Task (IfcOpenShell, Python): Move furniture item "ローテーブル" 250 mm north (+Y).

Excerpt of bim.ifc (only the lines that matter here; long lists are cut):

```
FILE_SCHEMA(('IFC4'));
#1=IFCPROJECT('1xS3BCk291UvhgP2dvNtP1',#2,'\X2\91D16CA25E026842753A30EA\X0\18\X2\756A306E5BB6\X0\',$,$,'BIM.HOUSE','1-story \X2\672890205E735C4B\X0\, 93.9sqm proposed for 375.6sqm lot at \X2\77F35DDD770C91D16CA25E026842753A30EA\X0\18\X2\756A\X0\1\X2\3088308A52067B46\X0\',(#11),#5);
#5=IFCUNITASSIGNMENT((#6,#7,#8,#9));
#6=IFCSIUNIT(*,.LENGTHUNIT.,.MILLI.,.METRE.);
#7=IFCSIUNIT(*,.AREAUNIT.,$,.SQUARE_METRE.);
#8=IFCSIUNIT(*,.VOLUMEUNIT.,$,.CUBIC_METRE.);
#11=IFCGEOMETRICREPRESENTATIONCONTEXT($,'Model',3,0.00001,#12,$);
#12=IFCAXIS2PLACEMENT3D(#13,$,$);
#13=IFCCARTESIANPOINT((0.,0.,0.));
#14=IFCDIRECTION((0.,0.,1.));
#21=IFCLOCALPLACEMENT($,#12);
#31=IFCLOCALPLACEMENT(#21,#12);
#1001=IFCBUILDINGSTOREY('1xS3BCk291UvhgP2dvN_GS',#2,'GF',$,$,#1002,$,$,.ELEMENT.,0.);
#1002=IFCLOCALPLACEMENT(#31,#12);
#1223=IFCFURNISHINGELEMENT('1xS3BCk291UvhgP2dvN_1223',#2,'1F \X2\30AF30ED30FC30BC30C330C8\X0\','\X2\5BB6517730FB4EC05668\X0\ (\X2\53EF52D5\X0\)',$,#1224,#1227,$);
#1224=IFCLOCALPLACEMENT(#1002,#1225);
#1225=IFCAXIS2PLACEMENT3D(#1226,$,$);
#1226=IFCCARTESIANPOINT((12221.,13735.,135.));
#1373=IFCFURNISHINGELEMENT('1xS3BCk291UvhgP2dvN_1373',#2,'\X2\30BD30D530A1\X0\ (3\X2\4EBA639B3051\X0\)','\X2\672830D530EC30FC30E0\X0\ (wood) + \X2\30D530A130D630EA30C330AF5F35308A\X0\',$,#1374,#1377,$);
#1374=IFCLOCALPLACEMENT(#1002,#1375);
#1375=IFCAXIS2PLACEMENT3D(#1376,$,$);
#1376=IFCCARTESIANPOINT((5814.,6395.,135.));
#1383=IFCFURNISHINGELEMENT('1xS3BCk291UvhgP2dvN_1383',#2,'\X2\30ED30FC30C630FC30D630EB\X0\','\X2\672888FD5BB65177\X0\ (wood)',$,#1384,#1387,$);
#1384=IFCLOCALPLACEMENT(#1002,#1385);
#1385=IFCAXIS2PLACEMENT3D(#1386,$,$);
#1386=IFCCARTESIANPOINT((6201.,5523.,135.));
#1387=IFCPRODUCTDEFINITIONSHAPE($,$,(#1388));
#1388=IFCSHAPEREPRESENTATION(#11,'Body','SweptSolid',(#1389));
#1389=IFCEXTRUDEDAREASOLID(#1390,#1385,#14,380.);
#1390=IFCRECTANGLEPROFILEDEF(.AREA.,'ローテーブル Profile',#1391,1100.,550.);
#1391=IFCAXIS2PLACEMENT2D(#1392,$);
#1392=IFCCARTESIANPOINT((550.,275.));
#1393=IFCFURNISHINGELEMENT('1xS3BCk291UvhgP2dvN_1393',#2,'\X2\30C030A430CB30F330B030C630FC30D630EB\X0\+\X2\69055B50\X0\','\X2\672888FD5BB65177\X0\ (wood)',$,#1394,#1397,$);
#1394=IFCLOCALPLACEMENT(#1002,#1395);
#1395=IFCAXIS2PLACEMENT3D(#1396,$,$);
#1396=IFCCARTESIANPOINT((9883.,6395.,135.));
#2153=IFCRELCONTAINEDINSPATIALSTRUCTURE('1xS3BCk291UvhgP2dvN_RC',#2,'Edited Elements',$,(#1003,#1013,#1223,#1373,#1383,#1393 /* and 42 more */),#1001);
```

```python
import ifcopenshell
import ifcopenshell.api.geometry
import ifcopenshell.util.placement
import ifcopenshell.util.unit

model = ifcopenshell.open("bim.ifc")
unit_scale = ifcopenshell.util.unit.calculate_unit_scale(model)

item = model.by_guid("1xS3BCk291UvhgP2dvN_1383")
matrix = ifcopenshell.util.placement.get_local_placement(item.ObjectPlacement)
matrix[1, 3] += 0.25 / unit_scale
ifcopenshell.api.geometry.edit_object_placement(model, product=item, matrix=matrix, is_si=False)

print(ifcopenshell.util.placement.get_local_placement(item.ObjectPlacement).round(3) + 0.0)

model.write("bim_edited.ifc")
```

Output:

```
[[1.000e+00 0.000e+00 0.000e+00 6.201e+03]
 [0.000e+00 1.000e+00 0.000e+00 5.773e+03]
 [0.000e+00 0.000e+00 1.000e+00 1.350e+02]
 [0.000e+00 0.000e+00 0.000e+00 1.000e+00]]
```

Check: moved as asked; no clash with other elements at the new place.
